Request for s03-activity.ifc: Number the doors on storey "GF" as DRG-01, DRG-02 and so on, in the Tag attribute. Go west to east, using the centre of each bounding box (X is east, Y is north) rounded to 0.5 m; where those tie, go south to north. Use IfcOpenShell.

First a look at what the model holds.

```python
import ifcopenshell
import ifcopenshell.util.element
import ifcopenshell.util.placement

model = ifcopenshell.open("s03-activity.ifc")
print(model.schema)
storey = next(s for s in model.by_type("IfcBuildingStorey") if s.Name == "GF")
doors = [e for e in ifcopenshell.util.element.get_decomposition(storey) if e.is_a("IfcDoor")]
for e in sorted(doors, key=lambda e: e.id()):
    origin = ifcopenshell.util.placement.get_local_placement(e.ObjectPlacement)[:3, 3]
    print(e.id(), e.Tag, e.Name, origin.round(2) + 0.0, sep=" | ")
```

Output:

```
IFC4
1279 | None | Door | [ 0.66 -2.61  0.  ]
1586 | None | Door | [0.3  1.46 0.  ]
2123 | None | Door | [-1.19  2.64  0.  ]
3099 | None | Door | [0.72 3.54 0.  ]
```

```python
import ifcopenshell
import ifcopenshell.geom
import ifcopenshell.util.element
import ifcopenshell.util.shape

model = ifcopenshell.open("s03-activity.ifc")
settings = ifcopenshell.geom.settings()
settings.set("use-world-coords", True)


def centre(element):
    shape = ifcopenshell.geom.create_shape(settings, element)
    return ifcopenshell.util.shape.get_bbox_centroid(shape.geometry)


storey = next(s for s in model.by_type("IfcBuildingStorey") if s.Name == "GF")
doors = [e for e in ifcopenshell.util.element.get_decomposition(storey) if e.is_a("IfcDoor")]

# Insertion points can sit at a corner or the storey origin, so sort by the geometry (in metres).
centres = {e: centre(e) for e in doors}
doors.sort(key=lambda e: (round(centres[e][0] / 0.5), centres[e][1]))

for i, e in enumerate(doors, start=1):
    number = f"DRG-{i:02d}"
    e.Tag = number
    print(e.id(), number)

model.write("s03-activity_edited.ifc")
```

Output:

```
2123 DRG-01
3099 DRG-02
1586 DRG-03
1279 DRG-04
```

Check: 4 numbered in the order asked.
